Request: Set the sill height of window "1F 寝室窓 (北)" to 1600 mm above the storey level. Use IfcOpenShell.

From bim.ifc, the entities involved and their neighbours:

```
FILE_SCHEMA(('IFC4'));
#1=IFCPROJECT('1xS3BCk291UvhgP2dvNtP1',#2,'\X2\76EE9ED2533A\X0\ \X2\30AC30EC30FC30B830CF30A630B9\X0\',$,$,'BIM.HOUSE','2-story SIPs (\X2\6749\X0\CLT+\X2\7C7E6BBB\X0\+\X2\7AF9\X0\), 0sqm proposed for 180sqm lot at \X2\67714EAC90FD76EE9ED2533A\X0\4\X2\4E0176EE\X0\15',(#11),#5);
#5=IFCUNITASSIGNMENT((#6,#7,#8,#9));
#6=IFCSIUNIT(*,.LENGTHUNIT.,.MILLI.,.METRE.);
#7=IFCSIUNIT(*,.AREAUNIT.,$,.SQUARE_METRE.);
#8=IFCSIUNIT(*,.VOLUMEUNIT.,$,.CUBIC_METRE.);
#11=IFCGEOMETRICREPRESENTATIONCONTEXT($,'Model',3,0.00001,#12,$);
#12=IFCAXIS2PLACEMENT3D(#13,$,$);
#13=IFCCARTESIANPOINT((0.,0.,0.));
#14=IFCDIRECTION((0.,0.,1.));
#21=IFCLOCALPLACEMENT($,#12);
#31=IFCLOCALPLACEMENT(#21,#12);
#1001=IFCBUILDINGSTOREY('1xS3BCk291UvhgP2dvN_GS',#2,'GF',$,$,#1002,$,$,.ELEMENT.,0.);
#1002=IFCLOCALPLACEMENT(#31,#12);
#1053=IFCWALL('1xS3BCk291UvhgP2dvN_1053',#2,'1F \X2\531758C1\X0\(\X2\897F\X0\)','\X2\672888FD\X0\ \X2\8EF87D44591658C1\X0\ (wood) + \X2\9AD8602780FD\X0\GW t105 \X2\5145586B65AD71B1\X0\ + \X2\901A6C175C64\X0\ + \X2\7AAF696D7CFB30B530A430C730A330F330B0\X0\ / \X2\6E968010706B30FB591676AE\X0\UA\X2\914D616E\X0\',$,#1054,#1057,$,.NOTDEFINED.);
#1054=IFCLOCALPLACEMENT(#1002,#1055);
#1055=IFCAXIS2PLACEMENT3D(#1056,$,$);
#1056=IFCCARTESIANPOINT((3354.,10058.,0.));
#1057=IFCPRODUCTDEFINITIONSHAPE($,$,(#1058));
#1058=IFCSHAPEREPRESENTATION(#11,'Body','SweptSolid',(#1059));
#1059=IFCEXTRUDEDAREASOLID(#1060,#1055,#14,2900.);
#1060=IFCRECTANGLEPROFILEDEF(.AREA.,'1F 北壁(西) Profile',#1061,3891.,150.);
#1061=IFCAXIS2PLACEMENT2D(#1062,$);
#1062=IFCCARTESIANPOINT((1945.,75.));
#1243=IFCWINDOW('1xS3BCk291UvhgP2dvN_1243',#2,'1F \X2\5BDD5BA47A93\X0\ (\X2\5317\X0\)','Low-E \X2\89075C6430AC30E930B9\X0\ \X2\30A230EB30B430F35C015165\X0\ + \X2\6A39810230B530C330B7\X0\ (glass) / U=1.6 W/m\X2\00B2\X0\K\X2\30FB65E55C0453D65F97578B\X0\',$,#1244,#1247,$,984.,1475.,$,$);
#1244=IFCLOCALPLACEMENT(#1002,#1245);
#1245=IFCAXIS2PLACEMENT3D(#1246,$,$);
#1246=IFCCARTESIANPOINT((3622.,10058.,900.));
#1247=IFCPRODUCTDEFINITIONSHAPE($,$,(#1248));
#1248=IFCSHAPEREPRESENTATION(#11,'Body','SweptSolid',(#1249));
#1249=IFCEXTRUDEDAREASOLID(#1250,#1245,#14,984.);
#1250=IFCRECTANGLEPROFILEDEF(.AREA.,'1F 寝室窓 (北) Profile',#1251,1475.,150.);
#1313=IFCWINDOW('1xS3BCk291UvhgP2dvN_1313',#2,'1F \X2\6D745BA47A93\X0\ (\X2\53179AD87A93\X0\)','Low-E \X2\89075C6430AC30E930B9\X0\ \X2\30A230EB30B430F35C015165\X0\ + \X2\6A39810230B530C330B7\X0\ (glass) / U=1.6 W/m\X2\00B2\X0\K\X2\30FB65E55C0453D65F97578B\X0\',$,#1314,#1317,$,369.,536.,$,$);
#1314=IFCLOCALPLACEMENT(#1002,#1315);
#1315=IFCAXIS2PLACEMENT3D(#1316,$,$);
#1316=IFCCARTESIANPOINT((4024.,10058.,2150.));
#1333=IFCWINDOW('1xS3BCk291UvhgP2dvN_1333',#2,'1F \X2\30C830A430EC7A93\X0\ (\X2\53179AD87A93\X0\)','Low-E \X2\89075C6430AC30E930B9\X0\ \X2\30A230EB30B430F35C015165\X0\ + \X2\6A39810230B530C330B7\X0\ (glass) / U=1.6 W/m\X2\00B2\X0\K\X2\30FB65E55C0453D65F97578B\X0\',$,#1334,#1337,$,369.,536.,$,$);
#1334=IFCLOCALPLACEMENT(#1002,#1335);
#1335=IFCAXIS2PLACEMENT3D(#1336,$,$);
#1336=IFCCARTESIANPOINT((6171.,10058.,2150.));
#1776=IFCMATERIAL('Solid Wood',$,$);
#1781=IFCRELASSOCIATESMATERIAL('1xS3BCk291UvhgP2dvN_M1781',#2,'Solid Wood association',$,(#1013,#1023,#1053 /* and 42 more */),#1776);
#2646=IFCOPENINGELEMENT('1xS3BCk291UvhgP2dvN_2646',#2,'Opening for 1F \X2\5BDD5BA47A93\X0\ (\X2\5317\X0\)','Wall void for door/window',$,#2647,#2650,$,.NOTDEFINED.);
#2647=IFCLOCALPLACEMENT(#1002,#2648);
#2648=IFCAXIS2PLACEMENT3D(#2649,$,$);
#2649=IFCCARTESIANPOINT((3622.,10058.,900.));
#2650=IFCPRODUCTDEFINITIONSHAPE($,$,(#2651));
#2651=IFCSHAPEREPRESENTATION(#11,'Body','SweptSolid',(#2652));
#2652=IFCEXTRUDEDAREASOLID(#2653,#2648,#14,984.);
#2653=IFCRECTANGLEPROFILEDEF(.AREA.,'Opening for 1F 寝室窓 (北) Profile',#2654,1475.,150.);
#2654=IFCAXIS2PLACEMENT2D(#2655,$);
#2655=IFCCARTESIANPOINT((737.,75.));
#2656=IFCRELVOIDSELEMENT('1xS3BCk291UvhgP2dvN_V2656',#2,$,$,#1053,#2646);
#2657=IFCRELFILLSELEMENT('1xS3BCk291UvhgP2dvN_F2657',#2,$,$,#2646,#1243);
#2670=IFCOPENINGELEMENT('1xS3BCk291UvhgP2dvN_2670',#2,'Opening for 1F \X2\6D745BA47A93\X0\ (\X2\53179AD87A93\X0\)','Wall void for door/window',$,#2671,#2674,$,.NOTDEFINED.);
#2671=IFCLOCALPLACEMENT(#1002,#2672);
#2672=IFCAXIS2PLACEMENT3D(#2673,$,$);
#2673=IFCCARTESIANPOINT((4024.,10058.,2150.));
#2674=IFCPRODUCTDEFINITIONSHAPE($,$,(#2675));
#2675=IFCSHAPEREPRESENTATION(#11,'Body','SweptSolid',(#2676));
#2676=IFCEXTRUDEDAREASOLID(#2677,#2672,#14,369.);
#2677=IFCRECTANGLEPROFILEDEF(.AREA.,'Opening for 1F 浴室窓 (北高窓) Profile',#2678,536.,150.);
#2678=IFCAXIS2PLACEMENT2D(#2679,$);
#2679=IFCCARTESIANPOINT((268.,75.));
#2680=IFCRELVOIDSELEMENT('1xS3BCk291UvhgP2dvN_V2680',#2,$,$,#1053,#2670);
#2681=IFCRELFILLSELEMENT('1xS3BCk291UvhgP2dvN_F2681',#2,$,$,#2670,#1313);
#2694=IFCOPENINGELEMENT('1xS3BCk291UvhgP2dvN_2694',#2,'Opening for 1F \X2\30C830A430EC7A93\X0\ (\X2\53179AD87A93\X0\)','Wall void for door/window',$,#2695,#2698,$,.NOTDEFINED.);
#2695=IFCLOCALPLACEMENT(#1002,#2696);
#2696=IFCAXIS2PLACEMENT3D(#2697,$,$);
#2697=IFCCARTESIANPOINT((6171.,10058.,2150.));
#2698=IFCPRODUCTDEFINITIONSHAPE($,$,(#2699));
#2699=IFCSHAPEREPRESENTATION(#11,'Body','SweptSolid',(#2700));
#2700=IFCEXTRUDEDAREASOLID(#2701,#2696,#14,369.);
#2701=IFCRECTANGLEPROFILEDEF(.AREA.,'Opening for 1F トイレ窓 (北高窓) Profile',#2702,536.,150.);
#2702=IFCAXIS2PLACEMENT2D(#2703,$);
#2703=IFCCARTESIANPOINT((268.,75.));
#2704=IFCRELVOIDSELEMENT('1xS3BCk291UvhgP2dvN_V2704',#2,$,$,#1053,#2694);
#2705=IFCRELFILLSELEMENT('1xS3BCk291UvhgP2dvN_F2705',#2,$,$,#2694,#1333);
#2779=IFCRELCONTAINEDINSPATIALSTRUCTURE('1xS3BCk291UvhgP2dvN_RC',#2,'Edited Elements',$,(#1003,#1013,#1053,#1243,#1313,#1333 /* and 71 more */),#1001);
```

```python
import numpy as np
import ifcopenshell
import ifcopenshell.api.geometry
import ifcopenshell.geom
import ifcopenshell.util.element
import ifcopenshell.util.placement
import ifcopenshell.util.shape
import ifcopenshell.util.unit

model = ifcopenshell.open("bim.ifc")
unit_scale = ifcopenshell.util.unit.calculate_unit_scale(model)

window = model.by_guid("1xS3BCk291UvhgP2dvN_1243")
opening = window.FillsVoids[0].RelatingOpeningElement
storey = ifcopenshell.util.element.get_container(window, ifc_class="IfcBuildingStorey")
level = ifcopenshell.util.placement.get_local_placement(storey.ObjectPlacement)[2, 3]

# The opening's origin need not be at the sill, so measure its lowest point.
shape = ifcopenshell.geom.create_shape(ifcopenshell.geom.settings(), opening)
bottom = ifcopenshell.util.shape.get_shape_bottom_elevation(shape, shape.geometry) / unit_scale
dz = level + 1.6 / unit_scale - bottom

shift = np.array([0.0, 0.0, dz])
# The window is not placed relative to its opening, so move both.
for product in (opening, window):
    matrix = ifcopenshell.util.placement.get_local_placement(product.ObjectPlacement)
    matrix[:3, 3] += shift
    ifcopenshell.api.geometry.edit_object_placement(model, product=product, matrix=matrix, is_si=False)

print(f"moved by {dz * unit_scale:+.3f} m")

model.write("bim-out.ifc")
```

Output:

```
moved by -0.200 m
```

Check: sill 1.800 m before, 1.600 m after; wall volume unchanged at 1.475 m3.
